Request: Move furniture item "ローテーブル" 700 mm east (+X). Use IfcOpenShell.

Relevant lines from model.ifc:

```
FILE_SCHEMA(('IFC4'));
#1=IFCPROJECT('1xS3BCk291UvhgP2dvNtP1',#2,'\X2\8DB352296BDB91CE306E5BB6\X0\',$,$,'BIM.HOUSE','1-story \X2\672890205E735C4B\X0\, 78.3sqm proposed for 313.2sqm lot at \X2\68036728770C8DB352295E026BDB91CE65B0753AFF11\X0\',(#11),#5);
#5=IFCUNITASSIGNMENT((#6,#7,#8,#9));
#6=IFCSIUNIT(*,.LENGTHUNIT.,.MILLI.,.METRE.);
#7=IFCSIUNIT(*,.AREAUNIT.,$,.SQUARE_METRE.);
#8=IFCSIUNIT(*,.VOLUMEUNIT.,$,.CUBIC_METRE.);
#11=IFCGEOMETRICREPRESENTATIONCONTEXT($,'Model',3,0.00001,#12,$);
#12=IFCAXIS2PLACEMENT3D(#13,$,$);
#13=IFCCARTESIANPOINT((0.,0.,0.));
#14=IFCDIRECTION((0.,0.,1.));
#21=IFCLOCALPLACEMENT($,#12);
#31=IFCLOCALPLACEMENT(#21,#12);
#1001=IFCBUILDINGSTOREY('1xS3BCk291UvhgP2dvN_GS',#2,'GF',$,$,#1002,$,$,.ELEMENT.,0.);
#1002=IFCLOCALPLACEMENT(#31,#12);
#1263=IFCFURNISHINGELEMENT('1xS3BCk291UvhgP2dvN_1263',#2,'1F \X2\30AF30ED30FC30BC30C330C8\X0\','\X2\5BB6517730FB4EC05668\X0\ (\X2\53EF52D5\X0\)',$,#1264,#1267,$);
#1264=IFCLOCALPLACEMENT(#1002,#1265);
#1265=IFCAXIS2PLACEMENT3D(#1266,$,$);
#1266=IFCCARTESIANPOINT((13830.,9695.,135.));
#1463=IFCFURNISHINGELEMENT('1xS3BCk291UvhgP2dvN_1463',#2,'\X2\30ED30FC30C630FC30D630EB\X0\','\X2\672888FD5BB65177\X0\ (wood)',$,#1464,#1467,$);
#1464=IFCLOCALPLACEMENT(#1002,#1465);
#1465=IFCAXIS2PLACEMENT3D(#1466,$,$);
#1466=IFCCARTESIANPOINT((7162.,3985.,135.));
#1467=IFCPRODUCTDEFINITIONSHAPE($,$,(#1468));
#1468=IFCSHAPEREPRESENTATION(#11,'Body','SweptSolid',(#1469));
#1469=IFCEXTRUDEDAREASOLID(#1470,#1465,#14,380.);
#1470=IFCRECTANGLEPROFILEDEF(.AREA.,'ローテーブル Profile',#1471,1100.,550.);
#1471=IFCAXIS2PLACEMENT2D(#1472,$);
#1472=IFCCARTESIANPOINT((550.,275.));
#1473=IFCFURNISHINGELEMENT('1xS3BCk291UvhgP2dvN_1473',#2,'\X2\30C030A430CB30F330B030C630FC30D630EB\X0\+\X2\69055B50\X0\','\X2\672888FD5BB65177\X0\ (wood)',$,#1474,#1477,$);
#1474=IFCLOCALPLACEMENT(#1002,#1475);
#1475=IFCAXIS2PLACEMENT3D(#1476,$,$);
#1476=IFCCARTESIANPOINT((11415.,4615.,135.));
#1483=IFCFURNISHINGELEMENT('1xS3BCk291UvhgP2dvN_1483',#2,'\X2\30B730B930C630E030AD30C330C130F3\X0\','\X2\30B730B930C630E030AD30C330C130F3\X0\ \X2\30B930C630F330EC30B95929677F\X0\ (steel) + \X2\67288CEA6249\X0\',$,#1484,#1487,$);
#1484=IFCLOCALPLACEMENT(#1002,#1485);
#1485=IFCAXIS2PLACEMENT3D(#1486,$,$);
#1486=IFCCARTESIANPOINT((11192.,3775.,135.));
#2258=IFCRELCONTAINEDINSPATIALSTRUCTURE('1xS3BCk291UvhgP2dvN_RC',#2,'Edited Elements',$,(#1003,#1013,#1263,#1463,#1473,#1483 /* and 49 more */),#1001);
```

```python
import ifcopenshell
import ifcopenshell.api.geometry
import ifcopenshell.util.placement

model = ifcopenshell.open("model.ifc")

item = model.by_guid("1xS3BCk291UvhgP2dvN_1463")
matrix = ifcopenshell.util.placement.get_local_placement(item.ObjectPlacement)
matrix[0, 3] += 700.0
ifcopenshell.api.geometry.edit_object_placement(model, product=item, matrix=matrix, is_si=False)

print(ifcopenshell.util.placement.get_local_placement(item.ObjectPlacement).round(3) + 0.0)

model.write("model_updated.ifc")
```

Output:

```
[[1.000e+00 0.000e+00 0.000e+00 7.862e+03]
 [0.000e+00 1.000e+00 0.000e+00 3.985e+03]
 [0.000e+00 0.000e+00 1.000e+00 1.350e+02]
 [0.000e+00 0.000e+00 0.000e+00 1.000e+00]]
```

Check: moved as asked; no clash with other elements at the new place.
